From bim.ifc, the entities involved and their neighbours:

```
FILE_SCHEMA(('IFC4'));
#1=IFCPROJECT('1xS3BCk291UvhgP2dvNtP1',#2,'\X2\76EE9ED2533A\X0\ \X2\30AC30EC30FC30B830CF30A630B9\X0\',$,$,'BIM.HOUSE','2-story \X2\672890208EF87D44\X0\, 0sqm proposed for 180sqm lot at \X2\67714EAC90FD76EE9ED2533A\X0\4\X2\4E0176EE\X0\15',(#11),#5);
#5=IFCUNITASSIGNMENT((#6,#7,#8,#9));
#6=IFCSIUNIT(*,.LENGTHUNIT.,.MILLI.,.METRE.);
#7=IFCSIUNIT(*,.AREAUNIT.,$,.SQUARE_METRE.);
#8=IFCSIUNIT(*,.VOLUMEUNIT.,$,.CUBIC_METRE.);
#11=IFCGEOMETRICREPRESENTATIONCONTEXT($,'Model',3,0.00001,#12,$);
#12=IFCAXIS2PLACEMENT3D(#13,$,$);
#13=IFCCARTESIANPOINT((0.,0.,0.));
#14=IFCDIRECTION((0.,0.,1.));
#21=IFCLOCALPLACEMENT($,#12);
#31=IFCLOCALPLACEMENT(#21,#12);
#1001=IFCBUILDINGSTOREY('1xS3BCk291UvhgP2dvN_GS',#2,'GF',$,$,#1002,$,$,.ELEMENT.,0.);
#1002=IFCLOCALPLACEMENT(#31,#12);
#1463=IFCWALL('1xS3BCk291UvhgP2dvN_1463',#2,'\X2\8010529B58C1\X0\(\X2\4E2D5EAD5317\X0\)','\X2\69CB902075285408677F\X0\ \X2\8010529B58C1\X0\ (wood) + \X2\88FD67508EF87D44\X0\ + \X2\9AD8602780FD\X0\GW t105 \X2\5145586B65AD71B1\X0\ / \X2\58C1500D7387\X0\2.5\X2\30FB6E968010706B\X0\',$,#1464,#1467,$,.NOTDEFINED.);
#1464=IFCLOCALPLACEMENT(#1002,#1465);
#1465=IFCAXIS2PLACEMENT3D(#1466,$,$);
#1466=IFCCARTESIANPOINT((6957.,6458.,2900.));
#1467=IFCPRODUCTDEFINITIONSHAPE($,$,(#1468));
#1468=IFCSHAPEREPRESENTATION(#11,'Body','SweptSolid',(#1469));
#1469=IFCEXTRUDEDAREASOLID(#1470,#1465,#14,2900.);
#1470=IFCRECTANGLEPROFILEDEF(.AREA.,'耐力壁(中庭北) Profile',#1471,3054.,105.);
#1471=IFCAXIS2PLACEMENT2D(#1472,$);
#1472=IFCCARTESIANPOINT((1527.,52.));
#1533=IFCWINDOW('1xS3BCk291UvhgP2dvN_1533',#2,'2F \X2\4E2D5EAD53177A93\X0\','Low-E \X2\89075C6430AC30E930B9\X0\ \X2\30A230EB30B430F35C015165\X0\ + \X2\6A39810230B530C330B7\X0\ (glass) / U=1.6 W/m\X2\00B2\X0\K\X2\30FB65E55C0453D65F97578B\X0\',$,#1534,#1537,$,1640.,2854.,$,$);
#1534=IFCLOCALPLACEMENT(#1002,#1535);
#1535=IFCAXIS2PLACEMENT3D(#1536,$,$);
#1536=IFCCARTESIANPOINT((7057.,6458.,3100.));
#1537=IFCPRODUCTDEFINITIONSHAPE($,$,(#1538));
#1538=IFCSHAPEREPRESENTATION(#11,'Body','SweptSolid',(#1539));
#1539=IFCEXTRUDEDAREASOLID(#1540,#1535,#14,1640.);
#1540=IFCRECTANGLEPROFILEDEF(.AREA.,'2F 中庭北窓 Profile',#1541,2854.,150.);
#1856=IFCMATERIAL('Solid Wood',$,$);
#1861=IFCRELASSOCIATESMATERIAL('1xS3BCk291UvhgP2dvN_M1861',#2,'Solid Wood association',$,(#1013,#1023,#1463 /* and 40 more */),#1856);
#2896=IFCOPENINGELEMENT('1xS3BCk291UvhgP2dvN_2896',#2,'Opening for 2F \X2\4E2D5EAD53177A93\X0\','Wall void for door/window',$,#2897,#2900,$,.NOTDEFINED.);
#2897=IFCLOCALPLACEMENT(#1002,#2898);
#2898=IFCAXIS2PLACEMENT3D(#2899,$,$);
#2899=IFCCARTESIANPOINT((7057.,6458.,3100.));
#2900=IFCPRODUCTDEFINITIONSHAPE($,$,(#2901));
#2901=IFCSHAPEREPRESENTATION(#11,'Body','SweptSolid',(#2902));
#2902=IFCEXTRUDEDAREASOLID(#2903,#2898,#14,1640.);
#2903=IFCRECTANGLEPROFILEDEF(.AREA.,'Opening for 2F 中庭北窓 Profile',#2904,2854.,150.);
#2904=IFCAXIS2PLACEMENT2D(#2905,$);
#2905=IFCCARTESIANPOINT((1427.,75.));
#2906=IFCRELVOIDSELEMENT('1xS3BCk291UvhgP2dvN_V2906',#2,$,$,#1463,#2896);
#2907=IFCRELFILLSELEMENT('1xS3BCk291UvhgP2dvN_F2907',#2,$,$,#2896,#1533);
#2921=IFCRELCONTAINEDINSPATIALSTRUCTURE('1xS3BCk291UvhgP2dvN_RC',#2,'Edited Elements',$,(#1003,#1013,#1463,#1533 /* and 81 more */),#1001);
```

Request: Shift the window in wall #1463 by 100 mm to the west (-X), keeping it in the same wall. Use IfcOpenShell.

```python
import ifcopenshell
import ifcopenshell.api.geometry
import ifcopenshell.util.placement
import ifcopenshell.util.unit

model = ifcopenshell.open("bim.ifc")
unit_scale = ifcopenshell.util.unit.calculate_unit_scale(model)

window = model.by_guid("1xS3BCk291UvhgP2dvN_1533")
opening = window.FillsVoids[0].RelatingOpeningElement
wall = opening.VoidsElements[0].RelatingBuildingElement

wall_matrix = ifcopenshell.util.placement.get_local_placement(wall.ObjectPlacement)
shift = wall_matrix[:3, 0] * -0.1 / unit_scale
before = ifcopenshell.util.placement.get_local_placement(window.ObjectPlacement)[:3, 3].copy()

# The window is not placed relative to its opening, so move both.
for product in (opening, window):
    matrix = ifcopenshell.util.placement.get_local_placement(product.ObjectPlacement)
    matrix[:3, 3] += shift
    ifcopenshell.api.geometry.edit_object_placement(model, product=product, matrix=matrix, is_si=False)

after = ifcopenshell.util.placement.get_local_placement(window.ObjectPlacement)[:3, 3]
print("window moved by", (after - before).round(3) + 0.0)

model.write("bim_rev.ifc")
```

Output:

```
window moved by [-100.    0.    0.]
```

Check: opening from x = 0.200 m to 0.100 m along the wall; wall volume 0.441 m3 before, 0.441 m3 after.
